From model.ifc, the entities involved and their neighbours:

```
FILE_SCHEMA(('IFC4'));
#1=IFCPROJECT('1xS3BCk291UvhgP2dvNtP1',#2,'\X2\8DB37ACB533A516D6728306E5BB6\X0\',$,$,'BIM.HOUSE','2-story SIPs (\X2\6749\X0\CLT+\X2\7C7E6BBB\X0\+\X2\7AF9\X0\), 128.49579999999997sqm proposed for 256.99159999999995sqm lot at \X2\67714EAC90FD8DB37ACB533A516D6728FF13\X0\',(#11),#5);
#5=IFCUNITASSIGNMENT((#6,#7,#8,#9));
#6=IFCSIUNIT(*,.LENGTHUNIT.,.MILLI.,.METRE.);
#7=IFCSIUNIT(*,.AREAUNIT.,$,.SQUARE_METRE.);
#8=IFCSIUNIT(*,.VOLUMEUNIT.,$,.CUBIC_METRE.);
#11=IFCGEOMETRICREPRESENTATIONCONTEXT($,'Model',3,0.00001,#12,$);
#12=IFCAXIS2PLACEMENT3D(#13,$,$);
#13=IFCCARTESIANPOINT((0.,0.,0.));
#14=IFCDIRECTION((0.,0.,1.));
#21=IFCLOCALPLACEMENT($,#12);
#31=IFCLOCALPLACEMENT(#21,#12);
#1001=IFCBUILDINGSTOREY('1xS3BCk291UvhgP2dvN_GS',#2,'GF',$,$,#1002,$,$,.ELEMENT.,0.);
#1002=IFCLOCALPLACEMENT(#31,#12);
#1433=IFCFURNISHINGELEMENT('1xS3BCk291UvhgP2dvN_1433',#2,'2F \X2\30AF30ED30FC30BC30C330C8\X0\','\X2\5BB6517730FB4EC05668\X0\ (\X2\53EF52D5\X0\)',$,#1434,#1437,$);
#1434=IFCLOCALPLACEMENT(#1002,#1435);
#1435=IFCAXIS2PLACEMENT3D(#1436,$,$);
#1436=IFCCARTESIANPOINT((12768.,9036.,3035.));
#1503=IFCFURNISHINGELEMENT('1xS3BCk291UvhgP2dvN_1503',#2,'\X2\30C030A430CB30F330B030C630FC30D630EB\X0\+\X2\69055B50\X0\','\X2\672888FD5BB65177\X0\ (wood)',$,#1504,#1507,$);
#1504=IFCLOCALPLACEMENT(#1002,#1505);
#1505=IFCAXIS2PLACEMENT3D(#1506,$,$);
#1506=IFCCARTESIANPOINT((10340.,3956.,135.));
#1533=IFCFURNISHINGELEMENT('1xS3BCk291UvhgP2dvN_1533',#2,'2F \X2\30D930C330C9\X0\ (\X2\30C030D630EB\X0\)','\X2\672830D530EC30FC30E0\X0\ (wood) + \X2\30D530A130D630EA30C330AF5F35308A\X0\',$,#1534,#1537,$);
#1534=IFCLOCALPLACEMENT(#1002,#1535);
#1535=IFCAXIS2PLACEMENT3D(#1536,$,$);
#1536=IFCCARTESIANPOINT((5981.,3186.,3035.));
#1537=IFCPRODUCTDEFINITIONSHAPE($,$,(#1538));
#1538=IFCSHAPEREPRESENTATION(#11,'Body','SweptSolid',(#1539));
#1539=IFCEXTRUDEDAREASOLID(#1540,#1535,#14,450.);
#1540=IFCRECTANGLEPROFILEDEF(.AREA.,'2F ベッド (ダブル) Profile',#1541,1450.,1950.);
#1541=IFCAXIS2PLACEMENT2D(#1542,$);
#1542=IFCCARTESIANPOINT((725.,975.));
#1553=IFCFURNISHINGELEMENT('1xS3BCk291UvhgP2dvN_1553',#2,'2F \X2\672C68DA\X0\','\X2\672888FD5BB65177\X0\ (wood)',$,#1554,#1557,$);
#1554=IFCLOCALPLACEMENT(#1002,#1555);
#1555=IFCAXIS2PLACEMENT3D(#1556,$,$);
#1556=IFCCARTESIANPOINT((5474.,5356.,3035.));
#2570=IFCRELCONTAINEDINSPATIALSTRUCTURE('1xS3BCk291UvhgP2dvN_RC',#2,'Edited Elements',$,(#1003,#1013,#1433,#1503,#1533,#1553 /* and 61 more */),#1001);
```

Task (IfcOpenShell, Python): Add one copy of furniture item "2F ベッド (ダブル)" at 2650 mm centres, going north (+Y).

```python
import numpy as np
import ifcopenshell
import ifcopenshell.api.geometry
import ifcopenshell.api.root
import ifcopenshell.util.element
import ifcopenshell.util.placement
import ifcopenshell.util.unit

model = ifcopenshell.open("model.ifc")
unit_scale = ifcopenshell.util.unit.calculate_unit_scale(model)


def reuse_history(source, copy):
    """copy_class also copies each property set's owner history, people and application; keep the originals."""
    for rel in copy.IsDefinedBy:
        if rel.is_a("IfcRelDefinesByProperties") and (history := rel.RelatingPropertyDefinition.OwnerHistory):
            rel.RelatingPropertyDefinition.OwnerHistory = source.OwnerHistory
            ifcopenshell.util.element.remove_deep2(model, history)


source = model.by_guid("1xS3BCk291UvhgP2dvN_1533")
base = ifcopenshell.util.placement.get_local_placement(source.ObjectPlacement)
step = np.array([0.0, 1.0, 0.0]) * 2.65 / unit_scale

for i in range(1, 2):
    copy = ifcopenshell.api.root.copy_class(model, product=source)
    copy.Representation = ifcopenshell.util.element.copy_deep(
        model, source.Representation, exclude=["IfcGeometricRepresentationContext", "IfcRepresentationMap"]
    )
    reuse_history(source, copy)
    matrix = base.copy()
    matrix[:3, 3] += i * step
    print("added at", matrix[:3, 3].round(3) + 0.0)
    ifcopenshell.api.geometry.edit_object_placement(model, product=copy, matrix=matrix, is_si=False)

model.write("model_updated.ifc")
```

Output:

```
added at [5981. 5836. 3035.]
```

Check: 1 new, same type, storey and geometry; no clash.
